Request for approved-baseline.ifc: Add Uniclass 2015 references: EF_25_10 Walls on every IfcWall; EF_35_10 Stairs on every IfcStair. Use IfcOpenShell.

First a look at what the model holds.

```python
import ifcopenshell

model = ifcopenshell.open("approved-baseline.ifc")
print(model.schema)
print("classifications:", [c.Name for c in model.by_type("IfcClassification")])
for ifc_class in ("IfcDoor", "IfcRoof", "IfcStair", "IfcWall", "IfcWindow"):
    print(ifc_class, len(model.by_type(ifc_class)))
```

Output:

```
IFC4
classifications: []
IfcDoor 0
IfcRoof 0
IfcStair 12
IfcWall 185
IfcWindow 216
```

```python
import ifcopenshell
import ifcopenshell.api.classification

model = ifcopenshell.open("approved-baseline.ifc")

system = ifcopenshell.api.classification.add_classification(model, classification="Uniclass 2015")

codes = {
    "IfcWall": ("EF_25_10", "Walls"),
    "IfcStair": ("EF_35_10", "Stairs"),
}
for ifc_class, (code, name) in codes.items():
    products = model.by_type(ifc_class)
    ifcopenshell.api.classification.add_reference(
        model, products=products, classification=system, identification=code, name=name
    )
    print(code, len(products))

model.write("approved-baseline_rev.ifc")
```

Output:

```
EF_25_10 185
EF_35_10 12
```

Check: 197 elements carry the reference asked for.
